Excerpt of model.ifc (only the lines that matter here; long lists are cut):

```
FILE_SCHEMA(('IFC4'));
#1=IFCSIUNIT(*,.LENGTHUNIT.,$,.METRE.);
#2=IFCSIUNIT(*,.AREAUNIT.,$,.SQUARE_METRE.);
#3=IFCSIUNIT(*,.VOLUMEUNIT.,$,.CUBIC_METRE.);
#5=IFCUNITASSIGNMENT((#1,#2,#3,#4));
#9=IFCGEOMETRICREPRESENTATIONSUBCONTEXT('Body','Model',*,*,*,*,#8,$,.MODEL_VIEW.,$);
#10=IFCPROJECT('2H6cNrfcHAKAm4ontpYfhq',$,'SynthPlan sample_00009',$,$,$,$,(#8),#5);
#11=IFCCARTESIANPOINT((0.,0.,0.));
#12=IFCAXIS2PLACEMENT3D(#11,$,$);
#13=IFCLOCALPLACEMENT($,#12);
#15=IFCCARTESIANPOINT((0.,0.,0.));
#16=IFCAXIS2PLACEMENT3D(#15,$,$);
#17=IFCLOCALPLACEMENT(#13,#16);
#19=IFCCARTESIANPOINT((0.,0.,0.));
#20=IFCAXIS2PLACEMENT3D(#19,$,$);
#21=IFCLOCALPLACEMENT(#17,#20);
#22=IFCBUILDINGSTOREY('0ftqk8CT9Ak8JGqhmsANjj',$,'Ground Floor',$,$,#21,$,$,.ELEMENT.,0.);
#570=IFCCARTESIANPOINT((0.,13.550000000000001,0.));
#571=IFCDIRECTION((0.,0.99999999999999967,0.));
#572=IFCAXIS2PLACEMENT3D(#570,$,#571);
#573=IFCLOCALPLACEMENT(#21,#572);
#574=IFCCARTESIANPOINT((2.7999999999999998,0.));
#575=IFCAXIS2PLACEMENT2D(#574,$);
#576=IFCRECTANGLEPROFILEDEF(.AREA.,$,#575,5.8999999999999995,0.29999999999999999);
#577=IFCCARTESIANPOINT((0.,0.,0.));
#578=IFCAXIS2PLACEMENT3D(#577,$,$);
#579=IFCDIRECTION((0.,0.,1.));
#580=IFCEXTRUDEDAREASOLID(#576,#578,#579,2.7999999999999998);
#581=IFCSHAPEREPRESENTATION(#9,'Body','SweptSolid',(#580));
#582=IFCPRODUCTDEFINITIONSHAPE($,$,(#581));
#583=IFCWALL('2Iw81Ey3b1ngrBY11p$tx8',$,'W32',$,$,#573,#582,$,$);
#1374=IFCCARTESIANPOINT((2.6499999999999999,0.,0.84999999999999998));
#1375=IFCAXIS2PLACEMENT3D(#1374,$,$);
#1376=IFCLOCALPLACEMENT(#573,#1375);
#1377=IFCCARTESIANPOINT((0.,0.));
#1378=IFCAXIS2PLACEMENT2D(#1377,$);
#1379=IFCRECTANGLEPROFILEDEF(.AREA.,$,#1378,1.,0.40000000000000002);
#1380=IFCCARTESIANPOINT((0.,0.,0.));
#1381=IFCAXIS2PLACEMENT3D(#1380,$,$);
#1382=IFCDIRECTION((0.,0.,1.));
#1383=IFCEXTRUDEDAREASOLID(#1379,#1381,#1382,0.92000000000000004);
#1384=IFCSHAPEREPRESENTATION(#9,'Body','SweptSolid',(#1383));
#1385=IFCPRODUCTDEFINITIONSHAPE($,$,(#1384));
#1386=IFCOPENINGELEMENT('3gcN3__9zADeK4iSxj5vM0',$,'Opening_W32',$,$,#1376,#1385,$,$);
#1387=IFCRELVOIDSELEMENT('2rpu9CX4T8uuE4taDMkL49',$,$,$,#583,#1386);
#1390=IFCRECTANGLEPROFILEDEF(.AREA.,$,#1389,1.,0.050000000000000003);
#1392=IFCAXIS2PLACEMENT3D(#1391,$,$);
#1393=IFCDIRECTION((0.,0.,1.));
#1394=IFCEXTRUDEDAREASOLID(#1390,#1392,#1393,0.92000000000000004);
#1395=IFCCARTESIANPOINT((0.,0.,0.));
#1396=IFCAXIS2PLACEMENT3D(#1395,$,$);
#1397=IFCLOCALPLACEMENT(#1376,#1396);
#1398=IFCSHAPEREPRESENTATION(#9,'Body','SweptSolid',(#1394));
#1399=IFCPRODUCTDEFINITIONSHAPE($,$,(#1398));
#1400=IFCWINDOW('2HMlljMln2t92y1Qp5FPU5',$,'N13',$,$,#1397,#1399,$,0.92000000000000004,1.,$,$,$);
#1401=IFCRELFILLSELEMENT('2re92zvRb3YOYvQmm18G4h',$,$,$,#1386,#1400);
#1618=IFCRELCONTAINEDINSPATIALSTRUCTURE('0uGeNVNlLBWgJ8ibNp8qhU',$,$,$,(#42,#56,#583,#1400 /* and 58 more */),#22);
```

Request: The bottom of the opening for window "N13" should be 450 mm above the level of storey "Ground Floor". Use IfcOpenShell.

```python
import numpy as np
import ifcopenshell
import ifcopenshell.api.geometry
import ifcopenshell.geom
import ifcopenshell.util.element
import ifcopenshell.util.placement
import ifcopenshell.util.shape
import ifcopenshell.util.unit

model = ifcopenshell.open("model.ifc")
unit_scale = ifcopenshell.util.unit.calculate_unit_scale(model)

window = model.by_guid("2HMlljMln2t92y1Qp5FPU5")
opening = window.FillsVoids[0].RelatingOpeningElement
storey = ifcopenshell.util.element.get_container(window, ifc_class="IfcBuildingStorey")
level = ifcopenshell.util.placement.get_local_placement(storey.ObjectPlacement)[2, 3]

# The opening's origin need not be at the sill, so measure its lowest point.
shape = ifcopenshell.geom.create_shape(ifcopenshell.geom.settings(), opening)
bottom = ifcopenshell.util.shape.get_shape_bottom_elevation(shape, shape.geometry) / unit_scale
dz = level + 0.45 / unit_scale - bottom

shift = np.array([0.0, 0.0, dz])
# The window is placed relative to its opening, so it follows when the opening moves.
matrix = ifcopenshell.util.placement.get_local_placement(opening.ObjectPlacement)
matrix[:3, 3] += shift
ifcopenshell.api.geometry.edit_object_placement(
    model, product=opening, matrix=matrix, is_si=False, should_transform_children=True
)

print(f"moved by {dz * unit_scale:+.3f} m")

model.write("model_edited.ifc")
```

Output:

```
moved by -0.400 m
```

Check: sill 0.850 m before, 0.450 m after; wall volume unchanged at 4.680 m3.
